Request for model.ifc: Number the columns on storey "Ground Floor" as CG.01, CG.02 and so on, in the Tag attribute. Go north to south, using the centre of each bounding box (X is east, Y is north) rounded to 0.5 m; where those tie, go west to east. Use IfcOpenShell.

First a look at what the model holds.

```python
import ifcopenshell
import ifcopenshell.util.element
import ifcopenshell.util.placement

model = ifcopenshell.open("model.ifc")
print(model.schema)
storey = next(s for s in model.by_type("IfcBuildingStorey") if s.Name == "Ground Floor")
columns = [e for e in ifcopenshell.util.element.get_decomposition(storey) if e.is_a("IfcColumn")]
for e in sorted(columns, key=lambda e: e.id()):
    origin = ifcopenshell.util.placement.get_local_placement(e.ObjectPlacement)[:3, 3]
    print(e.id(), e.Tag, e.Name, origin.round(2) + 0.0, sep=" | ")
```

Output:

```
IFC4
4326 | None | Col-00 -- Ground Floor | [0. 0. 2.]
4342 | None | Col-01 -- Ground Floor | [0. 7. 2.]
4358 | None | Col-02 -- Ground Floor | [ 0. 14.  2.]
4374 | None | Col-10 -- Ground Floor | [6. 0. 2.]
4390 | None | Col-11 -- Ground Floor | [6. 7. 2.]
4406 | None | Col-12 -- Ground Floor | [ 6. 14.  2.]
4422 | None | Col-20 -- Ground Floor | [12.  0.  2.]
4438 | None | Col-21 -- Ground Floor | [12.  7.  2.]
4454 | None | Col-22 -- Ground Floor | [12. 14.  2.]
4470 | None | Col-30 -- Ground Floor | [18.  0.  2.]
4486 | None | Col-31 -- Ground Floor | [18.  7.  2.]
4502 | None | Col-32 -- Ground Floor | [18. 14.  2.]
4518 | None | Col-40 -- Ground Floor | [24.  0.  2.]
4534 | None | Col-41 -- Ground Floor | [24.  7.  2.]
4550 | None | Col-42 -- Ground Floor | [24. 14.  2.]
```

```python
import ifcopenshell
import ifcopenshell.geom
import ifcopenshell.util.element
import ifcopenshell.util.shape

model = ifcopenshell.open("model.ifc")
settings = ifcopenshell.geom.settings()
settings.set("use-world-coords", True)


def centre(element):
    shape = ifcopenshell.geom.create_shape(settings, element)
    return ifcopenshell.util.shape.get_bbox_centroid(shape.geometry)


storey = next(s for s in model.by_type("IfcBuildingStorey") if s.Name == "Ground Floor")
columns = [e for e in ifcopenshell.util.element.get_decomposition(storey) if e.is_a("IfcColumn")]

# Insertion points can sit at a corner or the storey origin, so sort by the geometry (in metres).
centres = {e: centre(e) for e in columns}
columns.sort(key=lambda e: (-round(centres[e][1] / 0.5), centres[e][0]))

for i, e in enumerate(columns, start=1):
    number = f"CG.{i:02d}"
    e.Tag = number
    print(e.id(), number)

model.write("model_edited.ifc")
```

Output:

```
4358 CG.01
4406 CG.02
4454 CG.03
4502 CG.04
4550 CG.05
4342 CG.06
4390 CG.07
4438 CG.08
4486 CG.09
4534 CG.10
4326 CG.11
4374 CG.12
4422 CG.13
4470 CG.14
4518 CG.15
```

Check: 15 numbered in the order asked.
